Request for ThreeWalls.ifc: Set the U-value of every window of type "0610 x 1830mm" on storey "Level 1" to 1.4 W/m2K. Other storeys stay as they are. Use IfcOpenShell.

First a look at what the model holds.

```python
import ifcopenshell
import ifcopenshell.util.element

model = ifcopenshell.open("ThreeWalls.ifc")
print(model.schema)
storey = next(s for s in model.by_type("IfcBuildingStorey") if s.Name == "Level 1")
windows = [e for e in ifcopenshell.util.element.get_decomposition(storey) if e.is_a("IfcWindow")]
seen = {}
for e in windows:
    element_type = ifcopenshell.util.element.get_type(e)
    key = (element_type.Name if element_type != e and element_type else None, ifcopenshell.util.element.get_pset(e, "Pset_WindowCommon", "ThermalTransmittance"))
    seen[key] = seen.get(key, 0) + 1
for (name, value), count in sorted(seen.items(), key=str):
    print(count, "x", name, "|", value)
```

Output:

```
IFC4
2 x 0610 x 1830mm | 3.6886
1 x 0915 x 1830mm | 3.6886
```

```python
import ifcopenshell
import ifcopenshell.api.pset
import ifcopenshell.util.element

model = ifcopenshell.open("ThreeWalls.ifc")

storey = next(s for s in model.by_type("IfcBuildingStorey") if s.Name == "Level 1")
windows = [e for e in ifcopenshell.util.element.get_decomposition(storey) if e.is_a("IfcWindow")]

count = 0
for e in windows:
    element_type = ifcopenshell.util.element.get_type(e)
    if element_type in (None, e) or element_type.Name != "0610 x 1830mm":
        continue
    # add_pset returns the element's existing set when there is one.
    pset = ifcopenshell.api.pset.add_pset(model, product=e, name="Pset_WindowCommon")
    ifcopenshell.api.pset.edit_pset(model, pset=pset, properties={"ThermalTransmittance": 1.4})
    count += 1

print(count, "windows updated")

model.write("ThreeWalls_updated.ifc")
```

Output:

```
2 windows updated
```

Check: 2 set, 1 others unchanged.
